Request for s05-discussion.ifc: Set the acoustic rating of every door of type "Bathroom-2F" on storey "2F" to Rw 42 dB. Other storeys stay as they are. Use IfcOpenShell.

First a look at what the model holds.

```python
import ifcopenshell
import ifcopenshell.util.element

model = ifcopenshell.open("s05-discussion.ifc")
print(model.schema)
storey = next(s for s in model.by_type("IfcBuildingStorey") if s.Name == "2F")
doors = [e for e in ifcopenshell.util.element.get_decomposition(storey) if e.is_a("IfcDoor")]
seen = {}
for e in doors:
    element_type = ifcopenshell.util.element.get_type(e)
    key = (element_type.Name if element_type != e and element_type else None, ifcopenshell.util.element.get_pset(e, "Pset_DoorCommon", "AcousticRating"))
    seen[key] = seen.get(key, 0) + 1
for (name, value), count in sorted(seen.items(), key=str):
    print(count, "x", name, "|", value)
```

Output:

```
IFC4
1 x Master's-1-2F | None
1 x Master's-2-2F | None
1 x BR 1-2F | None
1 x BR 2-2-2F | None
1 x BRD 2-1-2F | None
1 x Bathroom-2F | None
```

```python
import ifcopenshell
import ifcopenshell.api.pset
import ifcopenshell.util.element

model = ifcopenshell.open("s05-discussion.ifc")

storey = next(s for s in model.by_type("IfcBuildingStorey") if s.Name == "2F")
doors = [e for e in ifcopenshell.util.element.get_decomposition(storey) if e.is_a("IfcDoor")]

count = 0
for e in doors:
    element_type = ifcopenshell.util.element.get_type(e)
    if element_type in (None, e) or element_type.Name != "Bathroom-2F":
        continue
    # add_pset returns the element's existing set when there is one.
    pset = ifcopenshell.api.pset.add_pset(model, product=e, name="Pset_DoorCommon")
    ifcopenshell.api.pset.edit_pset(model, pset=pset, properties={"AcousticRating": "Rw 42 dB"})
    count += 1

print(count, "doors updated")

model.write("s05-discussion_v2.ifc")
```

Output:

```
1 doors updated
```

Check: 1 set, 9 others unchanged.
